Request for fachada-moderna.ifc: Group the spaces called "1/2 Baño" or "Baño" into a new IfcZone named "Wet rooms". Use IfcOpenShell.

First a look at what the model holds.

```python
import ifcopenshell

model = ifcopenshell.open("fachada-moderna.ifc")
print(model.schema)
seen = {}
for space in model.by_type("IfcSpace"):
    seen[space.LongName] = seen.get(space.LongName, 0) + 1
for name, count in sorted(seen.items(), key=str):
    print(count, "x", name)
print("zones:", [z.Name for z in model.by_type("IfcZone")][:20])
```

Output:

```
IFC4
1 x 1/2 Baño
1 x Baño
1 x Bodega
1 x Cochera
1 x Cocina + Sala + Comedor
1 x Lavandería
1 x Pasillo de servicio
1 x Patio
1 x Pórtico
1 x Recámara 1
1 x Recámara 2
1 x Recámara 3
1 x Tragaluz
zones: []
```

```python
import ifcopenshell
import ifcopenshell.api.group
import ifcopenshell.api.root

model = ifcopenshell.open("fachada-moderna.ifc")

names = {"1/2 Baño", "Baño"}
spaces = [s for s in model.by_type("IfcSpace") if s.LongName in names]

zone = ifcopenshell.api.root.create_entity(model, ifc_class="IfcZone", name="Wet rooms")
ifcopenshell.api.group.assign_group(model, products=spaces, group=zone)
print(len(spaces), "spaces in", zone.Name)

model.write("fachada-moderna_rev.ifc")
```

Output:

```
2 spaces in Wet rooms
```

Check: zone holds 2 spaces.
